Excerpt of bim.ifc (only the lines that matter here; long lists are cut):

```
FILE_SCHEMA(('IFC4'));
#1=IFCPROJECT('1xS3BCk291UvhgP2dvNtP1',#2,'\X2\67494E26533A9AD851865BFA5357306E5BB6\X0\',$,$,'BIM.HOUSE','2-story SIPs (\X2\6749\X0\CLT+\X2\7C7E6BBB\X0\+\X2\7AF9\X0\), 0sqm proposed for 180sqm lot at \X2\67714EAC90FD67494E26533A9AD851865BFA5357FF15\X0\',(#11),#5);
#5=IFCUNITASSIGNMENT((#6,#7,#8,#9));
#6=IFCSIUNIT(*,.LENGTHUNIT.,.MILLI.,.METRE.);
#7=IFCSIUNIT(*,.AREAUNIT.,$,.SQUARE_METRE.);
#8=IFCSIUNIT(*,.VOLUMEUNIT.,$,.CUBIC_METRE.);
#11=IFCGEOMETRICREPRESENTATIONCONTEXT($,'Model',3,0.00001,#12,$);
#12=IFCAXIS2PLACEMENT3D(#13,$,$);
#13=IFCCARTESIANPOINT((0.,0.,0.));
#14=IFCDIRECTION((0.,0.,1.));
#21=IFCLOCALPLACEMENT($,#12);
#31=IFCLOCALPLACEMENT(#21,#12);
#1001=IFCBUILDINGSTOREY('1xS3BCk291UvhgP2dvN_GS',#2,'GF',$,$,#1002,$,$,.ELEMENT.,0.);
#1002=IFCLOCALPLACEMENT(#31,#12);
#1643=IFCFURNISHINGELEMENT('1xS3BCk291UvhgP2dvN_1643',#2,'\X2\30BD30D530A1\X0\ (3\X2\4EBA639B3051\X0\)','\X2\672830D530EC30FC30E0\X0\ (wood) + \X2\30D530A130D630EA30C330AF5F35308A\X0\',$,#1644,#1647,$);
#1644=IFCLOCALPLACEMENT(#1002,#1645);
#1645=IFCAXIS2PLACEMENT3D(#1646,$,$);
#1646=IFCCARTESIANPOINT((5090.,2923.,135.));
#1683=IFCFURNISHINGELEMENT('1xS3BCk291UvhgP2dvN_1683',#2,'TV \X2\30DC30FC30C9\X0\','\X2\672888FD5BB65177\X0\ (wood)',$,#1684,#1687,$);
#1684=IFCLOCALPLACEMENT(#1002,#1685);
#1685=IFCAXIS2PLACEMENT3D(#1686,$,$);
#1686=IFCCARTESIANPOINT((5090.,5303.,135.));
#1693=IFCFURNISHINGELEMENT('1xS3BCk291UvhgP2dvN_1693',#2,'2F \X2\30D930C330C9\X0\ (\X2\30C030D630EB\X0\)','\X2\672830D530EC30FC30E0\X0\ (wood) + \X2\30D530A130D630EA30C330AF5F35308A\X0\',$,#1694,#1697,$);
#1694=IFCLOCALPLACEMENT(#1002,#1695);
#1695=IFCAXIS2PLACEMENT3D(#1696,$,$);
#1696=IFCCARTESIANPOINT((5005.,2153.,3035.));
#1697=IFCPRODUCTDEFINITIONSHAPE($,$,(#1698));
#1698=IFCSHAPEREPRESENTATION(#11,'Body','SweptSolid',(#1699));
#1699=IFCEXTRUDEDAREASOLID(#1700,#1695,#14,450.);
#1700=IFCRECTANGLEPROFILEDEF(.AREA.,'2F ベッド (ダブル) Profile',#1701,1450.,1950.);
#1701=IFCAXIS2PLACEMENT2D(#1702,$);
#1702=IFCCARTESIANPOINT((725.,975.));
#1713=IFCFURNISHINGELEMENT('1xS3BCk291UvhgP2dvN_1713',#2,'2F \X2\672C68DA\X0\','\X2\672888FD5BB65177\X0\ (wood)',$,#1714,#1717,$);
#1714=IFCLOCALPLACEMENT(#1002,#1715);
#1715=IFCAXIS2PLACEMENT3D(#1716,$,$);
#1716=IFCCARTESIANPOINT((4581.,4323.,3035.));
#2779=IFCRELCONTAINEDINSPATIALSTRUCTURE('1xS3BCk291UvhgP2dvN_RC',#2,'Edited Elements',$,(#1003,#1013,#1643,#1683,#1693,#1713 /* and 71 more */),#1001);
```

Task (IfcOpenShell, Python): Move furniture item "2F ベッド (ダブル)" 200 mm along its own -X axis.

```python
import ifcopenshell
import ifcopenshell.api.geometry
import ifcopenshell.util.placement
import ifcopenshell.util.unit

model = ifcopenshell.open("bim.ifc")
unit_scale = ifcopenshell.util.unit.calculate_unit_scale(model)

item = model.by_guid("1xS3BCk291UvhgP2dvN_1693")
matrix = ifcopenshell.util.placement.get_local_placement(item.ObjectPlacement)
matrix[:3, 3] -= matrix[:3, 0] * 0.2 / unit_scale
ifcopenshell.api.geometry.edit_object_placement(model, product=item, matrix=matrix, is_si=False)

print(ifcopenshell.util.placement.get_local_placement(item.ObjectPlacement).round(3) + 0.0)

model.write("bim_v2.ifc")
```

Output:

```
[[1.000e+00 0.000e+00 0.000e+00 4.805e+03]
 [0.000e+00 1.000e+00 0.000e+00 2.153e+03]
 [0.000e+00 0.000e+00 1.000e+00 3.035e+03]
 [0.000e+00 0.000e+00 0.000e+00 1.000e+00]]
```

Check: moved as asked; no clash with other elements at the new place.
